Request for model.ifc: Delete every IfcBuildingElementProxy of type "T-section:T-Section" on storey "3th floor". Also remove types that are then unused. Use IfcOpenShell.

First a look at what the model holds.

```python
import ifcopenshell
import ifcopenshell.util.element

model = ifcopenshell.open("model.ifc")
print(model.schema)
storey = next(s for s in model.by_type("IfcBuildingStorey") if s.Name == "3th floor")
proxies = [e for e in ifcopenshell.util.element.get_decomposition(storey) if e.is_a("IfcBuildingElementProxy")]
seen = {}
for e in proxies:
    element_type = ifcopenshell.util.element.get_type(e)
    name = element_type.Name if element_type not in (None, e) else None
    seen[name] = seen.get(name, 0) + 1
for name, count in sorted(seen.items(), key=str):
    print(count, "x", name)
```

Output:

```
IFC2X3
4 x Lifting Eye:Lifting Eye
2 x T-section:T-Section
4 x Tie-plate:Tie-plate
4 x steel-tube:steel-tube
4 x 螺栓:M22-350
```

```python
import ifcopenshell
import ifcopenshell.api.root
import ifcopenshell.util.element

model = ifcopenshell.open("model.ifc")

storey = next(s for s in model.by_type("IfcBuildingStorey") if s.Name == "3th floor")
proxies = [e for e in ifcopenshell.util.element.get_decomposition(storey) if e.is_a("IfcBuildingElementProxy")]
targets = [e for e in proxies if (t := ifcopenshell.util.element.get_type(e)) not in (None, e) and t.Name == "T-section:T-Section"]
types = {ifcopenshell.util.element.get_type(e) for e in targets} - {None, *targets}

for e in targets:
    ifcopenshell.api.root.remove_product(model, product=e)
print(len(targets), "removed")

unused = [t for t in types if not ifcopenshell.util.element.get_types(t)]
for t in unused:
    ifcopenshell.api.root.remove_product(model, product=t)
print(len(unused), "unused types removed")

model.write("model_v2.ifc")
```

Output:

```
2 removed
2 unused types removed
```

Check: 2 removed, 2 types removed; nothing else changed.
